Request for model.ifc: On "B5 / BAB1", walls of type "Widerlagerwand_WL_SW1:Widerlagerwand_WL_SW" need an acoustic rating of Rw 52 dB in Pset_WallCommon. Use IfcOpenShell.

First a look at what the model holds.

```python
import ifcopenshell
import ifcopenshell.util.element

model = ifcopenshell.open("model.ifc")
print(model.schema)
storey = next(s for s in model.by_type("IfcBuildingStorey") if s.Name == "B5 / BAB1")
walls = [e for e in ifcopenshell.util.element.get_decomposition(storey) if e.is_a("IfcWall")]
seen = {}
for e in walls:
    element_type = ifcopenshell.util.element.get_type(e)
    key = (element_type.Name if element_type != e and element_type else None, ifcopenshell.util.element.get_pset(e, "Pset_WallCommon", "AcousticRating"))
    seen[key] = seen.get(key, 0) + 1
for (name, value), count in sorted(seen.items(), key=str):
    print(count, "x", name, "|", value)
```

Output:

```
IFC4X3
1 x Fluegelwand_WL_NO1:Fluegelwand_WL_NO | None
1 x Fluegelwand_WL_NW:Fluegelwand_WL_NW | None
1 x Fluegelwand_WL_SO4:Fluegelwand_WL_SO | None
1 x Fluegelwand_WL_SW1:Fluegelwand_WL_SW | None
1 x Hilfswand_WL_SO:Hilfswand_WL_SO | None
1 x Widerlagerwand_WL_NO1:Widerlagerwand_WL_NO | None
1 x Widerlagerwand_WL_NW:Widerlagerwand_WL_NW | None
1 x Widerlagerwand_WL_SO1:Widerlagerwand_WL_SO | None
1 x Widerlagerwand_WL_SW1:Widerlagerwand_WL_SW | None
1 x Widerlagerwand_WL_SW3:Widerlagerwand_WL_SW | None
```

```python
import ifcopenshell
import ifcopenshell.api.pset
import ifcopenshell.util.element

model = ifcopenshell.open("model.ifc")

storey = next(s for s in model.by_type("IfcBuildingStorey") if s.Name == "B5 / BAB1")
walls = [e for e in ifcopenshell.util.element.get_decomposition(storey) if e.is_a("IfcWall")]

count = 0
for e in walls:
    element_type = ifcopenshell.util.element.get_type(e)
    if element_type in (None, e) or element_type.Name != "Widerlagerwand_WL_SW1:Widerlagerwand_WL_SW":
        continue
    # add_pset returns the element's existing set when there is one.
    pset = ifcopenshell.api.pset.add_pset(model, product=e, name="Pset_WallCommon")
    ifcopenshell.api.pset.edit_pset(model, pset=pset, properties={"AcousticRating": "Rw 52 dB"})
    count += 1

print(count, "walls updated")

model.write("model_v2.ifc")
```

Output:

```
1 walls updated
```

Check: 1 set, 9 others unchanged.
